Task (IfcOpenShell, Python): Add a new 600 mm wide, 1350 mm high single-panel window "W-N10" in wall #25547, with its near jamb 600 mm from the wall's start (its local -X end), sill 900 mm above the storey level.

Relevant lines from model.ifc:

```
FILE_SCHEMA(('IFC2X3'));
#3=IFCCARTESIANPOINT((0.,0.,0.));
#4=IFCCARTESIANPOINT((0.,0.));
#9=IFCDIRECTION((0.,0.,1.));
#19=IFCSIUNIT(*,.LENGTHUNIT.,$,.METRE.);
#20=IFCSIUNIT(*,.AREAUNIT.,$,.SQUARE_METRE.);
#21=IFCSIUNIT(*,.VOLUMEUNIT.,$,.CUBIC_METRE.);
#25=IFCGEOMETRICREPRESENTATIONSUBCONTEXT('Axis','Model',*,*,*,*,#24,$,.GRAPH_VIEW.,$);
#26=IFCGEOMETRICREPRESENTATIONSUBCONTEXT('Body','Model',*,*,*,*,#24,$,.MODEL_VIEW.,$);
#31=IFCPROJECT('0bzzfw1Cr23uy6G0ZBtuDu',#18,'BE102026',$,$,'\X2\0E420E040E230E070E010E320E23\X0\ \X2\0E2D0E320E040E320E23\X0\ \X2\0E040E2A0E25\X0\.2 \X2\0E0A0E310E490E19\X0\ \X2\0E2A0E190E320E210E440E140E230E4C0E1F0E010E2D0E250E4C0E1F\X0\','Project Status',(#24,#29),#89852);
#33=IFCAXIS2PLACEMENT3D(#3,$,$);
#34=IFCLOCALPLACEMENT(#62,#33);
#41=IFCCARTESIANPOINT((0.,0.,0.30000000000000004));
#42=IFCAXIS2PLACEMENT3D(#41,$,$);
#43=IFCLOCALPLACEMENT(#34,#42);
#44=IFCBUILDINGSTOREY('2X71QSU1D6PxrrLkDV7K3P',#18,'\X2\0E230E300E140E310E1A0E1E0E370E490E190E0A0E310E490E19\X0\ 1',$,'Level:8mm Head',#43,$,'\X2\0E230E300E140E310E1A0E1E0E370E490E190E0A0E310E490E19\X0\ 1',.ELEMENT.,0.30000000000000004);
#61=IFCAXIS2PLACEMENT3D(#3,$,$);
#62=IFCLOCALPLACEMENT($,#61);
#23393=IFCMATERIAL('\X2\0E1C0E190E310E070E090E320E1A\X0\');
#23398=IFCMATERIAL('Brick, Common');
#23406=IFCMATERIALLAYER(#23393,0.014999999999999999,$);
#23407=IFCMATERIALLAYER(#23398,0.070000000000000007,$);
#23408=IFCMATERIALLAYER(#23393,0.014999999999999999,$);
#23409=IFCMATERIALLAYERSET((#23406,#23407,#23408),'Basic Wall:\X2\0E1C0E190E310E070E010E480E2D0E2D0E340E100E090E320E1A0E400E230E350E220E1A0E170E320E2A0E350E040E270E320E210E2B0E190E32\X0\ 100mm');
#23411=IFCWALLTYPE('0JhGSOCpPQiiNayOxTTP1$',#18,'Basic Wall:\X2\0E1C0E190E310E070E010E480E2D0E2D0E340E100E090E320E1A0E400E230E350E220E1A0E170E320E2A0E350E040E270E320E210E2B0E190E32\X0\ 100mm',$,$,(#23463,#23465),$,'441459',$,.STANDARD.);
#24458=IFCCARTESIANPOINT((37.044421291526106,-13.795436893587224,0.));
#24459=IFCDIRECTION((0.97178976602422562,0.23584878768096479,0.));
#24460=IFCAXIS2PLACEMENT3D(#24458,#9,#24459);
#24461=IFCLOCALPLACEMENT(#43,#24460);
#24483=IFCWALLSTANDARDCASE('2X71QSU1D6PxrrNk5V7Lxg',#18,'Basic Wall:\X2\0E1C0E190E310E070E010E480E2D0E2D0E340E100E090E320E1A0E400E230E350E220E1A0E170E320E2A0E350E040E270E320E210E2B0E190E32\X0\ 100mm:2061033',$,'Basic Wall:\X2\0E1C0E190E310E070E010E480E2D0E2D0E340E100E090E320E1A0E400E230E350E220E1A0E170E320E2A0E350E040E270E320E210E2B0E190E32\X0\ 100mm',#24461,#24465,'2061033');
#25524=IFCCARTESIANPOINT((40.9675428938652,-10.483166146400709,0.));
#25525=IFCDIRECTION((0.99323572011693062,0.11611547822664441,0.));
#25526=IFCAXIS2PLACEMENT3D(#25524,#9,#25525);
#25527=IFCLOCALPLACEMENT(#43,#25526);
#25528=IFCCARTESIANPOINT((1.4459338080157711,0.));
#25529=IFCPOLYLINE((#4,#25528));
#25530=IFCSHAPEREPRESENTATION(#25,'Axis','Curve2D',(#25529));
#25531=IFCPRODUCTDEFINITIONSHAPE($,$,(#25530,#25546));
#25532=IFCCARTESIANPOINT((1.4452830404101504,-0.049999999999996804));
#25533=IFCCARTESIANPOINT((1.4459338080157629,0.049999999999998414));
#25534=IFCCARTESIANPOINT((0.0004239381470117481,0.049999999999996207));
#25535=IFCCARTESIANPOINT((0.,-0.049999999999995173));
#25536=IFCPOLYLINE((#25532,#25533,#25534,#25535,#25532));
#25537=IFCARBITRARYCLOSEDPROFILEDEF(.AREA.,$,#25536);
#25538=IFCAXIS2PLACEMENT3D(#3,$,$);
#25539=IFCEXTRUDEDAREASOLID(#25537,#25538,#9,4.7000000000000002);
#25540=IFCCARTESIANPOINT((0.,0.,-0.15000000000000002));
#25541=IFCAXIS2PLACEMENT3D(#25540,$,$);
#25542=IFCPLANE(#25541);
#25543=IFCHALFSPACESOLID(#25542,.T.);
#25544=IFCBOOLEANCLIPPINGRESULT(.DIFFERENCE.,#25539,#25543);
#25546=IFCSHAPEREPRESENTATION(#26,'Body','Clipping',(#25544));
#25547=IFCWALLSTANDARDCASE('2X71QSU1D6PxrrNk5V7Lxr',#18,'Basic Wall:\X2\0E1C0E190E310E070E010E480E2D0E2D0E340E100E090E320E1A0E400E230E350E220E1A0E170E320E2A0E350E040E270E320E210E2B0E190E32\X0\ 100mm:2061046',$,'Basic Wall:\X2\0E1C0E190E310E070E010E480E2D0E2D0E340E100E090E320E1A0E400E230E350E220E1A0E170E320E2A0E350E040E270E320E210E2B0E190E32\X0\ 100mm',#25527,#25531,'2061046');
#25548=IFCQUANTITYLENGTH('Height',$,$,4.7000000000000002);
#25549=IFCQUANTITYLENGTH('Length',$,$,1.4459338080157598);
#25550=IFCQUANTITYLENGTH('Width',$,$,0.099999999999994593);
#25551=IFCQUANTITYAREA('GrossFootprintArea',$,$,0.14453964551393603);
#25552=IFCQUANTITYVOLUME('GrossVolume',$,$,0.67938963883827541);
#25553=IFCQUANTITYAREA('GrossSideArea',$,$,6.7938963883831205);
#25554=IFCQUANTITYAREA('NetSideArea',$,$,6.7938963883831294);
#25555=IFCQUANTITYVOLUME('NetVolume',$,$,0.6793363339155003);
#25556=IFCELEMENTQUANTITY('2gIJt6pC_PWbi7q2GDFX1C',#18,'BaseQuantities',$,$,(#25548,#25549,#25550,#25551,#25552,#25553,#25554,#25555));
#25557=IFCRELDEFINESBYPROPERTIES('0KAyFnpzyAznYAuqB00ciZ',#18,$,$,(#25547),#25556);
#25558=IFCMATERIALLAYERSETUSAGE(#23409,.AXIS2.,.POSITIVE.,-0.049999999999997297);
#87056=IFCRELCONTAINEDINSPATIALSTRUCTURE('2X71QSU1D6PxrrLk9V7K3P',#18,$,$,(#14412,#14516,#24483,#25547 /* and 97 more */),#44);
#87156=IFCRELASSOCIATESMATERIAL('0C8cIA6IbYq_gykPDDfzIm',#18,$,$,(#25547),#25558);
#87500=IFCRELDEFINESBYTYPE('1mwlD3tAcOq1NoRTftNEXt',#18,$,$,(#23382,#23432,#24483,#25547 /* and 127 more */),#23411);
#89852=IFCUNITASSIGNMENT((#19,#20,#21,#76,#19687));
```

```python
import numpy as np
import ifcopenshell
import ifcopenshell.api.feature
import ifcopenshell.api.geometry
import ifcopenshell.api.pset
import ifcopenshell.api.root
import ifcopenshell.api.spatial
import ifcopenshell.api.type
import ifcopenshell.geom
import ifcopenshell.util.element
import ifcopenshell.util.placement
import ifcopenshell.util.representation
import ifcopenshell.util.shape
import ifcopenshell.util.unit

model = ifcopenshell.open("model.ifc")
unit_scale = ifcopenshell.util.unit.calculate_unit_scale(model)
area_scale = ifcopenshell.util.unit.calculate_unit_scale(model, "AREAUNIT")
volume_scale = ifcopenshell.util.unit.calculate_unit_scale(model, "VOLUMEUNIT")
settings = ifcopenshell.geom.settings()


def volume(element):
    """Net volume in cubic metres, openings subtracted."""
    shape = ifcopenshell.geom.create_shape(settings, element)
    return ifcopenshell.util.shape.get_volume(shape.geometry)


wall = model.by_id(25547)
storey = ifcopenshell.util.element.get_container(wall, ifc_class="IfcBuildingStorey")
context = ifcopenshell.util.representation.get_context(model, "Model", "Body", "MODEL_VIEW")
before = volume(wall)

width, height, from_end, sill = 0.6, 1.35, 0.6, 0.9  # metres

# The wall runs along its own X axis, and the end named is its -X end.
wall_shape = ifcopenshell.geom.create_shape(settings, wall)
x, y, z = ifcopenshell.util.shape.get_vertices(wall_shape.geometry).T
start = x.min() + from_end
face, thickness = float(y.min()), float(y.max() - y.min())
wall_matrix = ifcopenshell.util.placement.get_local_placement(wall.ObjectPlacement)
level = ifcopenshell.util.placement.get_local_placement(storey.ObjectPlacement)[2, 3]


def in_wall(x, y):
    """Placement at x, y metres in the wall's axes, at sill height."""
    matrix = wall_matrix.copy()
    matrix[:, 3] = wall_matrix @ np.array([x / unit_scale, y / unit_scale, 0.0, 1.0])
    matrix[2, 3] = level + sill / unit_scale
    return matrix


# Opening: a box that overshoots both wall faces by 50 mm.
opening = ifcopenshell.api.root.create_entity(model, ifc_class="IfcOpeningElement")
box = ifcopenshell.api.geometry.add_wall_representation(
    model, context=context, length=width, height=height, thickness=thickness + 0.1
)
ifcopenshell.api.geometry.assign_representation(model, product=opening, representation=box)
ifcopenshell.api.geometry.edit_object_placement(model, product=opening, matrix=in_wall(start, face - 0.05), is_si=False)
ifcopenshell.api.feature.add_feature(model, feature=opening, element=wall)

window = ifcopenshell.api.root.create_entity(model, ifc_class="IfcWindow", name="W-N10")
window.OverallWidth, window.OverallHeight = width / unit_scale, height / unit_scale
body = ifcopenshell.api.geometry.add_window_representation(
    model,
    context=context,
    overall_width=window.OverallWidth,
    overall_height=window.OverallHeight,
    partition_type="SINGLE_PANEL",
)
ifcopenshell.api.geometry.assign_representation(model, product=window, representation=body)
ifcopenshell.api.spatial.assign_container(model, products=[window], relating_structure=storey)
fills = ifcopenshell.api.feature.add_filling(model, opening=opening, element=window)
fills.OwnerHistory = window.OwnerHistory  # required in IFC2X3

# IFC2X3 keeps the operation on the window style.
style = ifcopenshell.api.root.create_entity(model, ifc_class="IfcWindowStyle", name="W-N10")
style.OperationType, style.ConstructionType = "SINGLE_PANEL", "NOTDEFINED"
style.ParameterTakesPrecedence = style.Sizeable = False
ifcopenshell.api.type.assign_type(model, related_objects=[window], relating_type=style)

# Centre the window in the wall's thickness.
ifcopenshell.api.geometry.edit_object_placement(model, product=window, matrix=in_wall(start, face), is_si=False)
window_shape = ifcopenshell.geom.create_shape(settings, window)
depth = ifcopenshell.util.shape.get_vertices(window_shape.geometry)[:, 1]
offset = face + thickness / 2 - (depth.min() + depth.max()) / 2
ifcopenshell.api.geometry.edit_object_placement(model, product=window, matrix=in_wall(start, offset), is_si=False)

after = volume(wall)

# Update the wall's stored quantities.
qto = model.by_id(ifcopenshell.util.element.get_pset(wall, "BaseQuantities", should_inherit=False)["id"])
ifcopenshell.api.pset.edit_qto(model, qto=qto, properties={
    "NetSideArea": after / thickness / area_scale,
    "NetVolume": after / volume_scale,
})

print(f"wall volume {before:.3f} -> {after:.3f} m3")

model.write("model_rev.ifc")
```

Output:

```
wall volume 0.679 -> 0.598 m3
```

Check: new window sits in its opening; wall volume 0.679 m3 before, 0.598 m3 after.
